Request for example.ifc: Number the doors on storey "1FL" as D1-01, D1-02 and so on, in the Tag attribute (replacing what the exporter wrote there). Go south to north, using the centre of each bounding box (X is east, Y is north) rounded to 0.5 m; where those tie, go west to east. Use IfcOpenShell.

First a look at what the model holds.

```python
import ifcopenshell
import ifcopenshell.util.element
import ifcopenshell.util.placement

model = ifcopenshell.open("example.ifc")
print(model.schema)
storey = next(s for s in model.by_type("IfcBuildingStorey") if s.Name == "1FL")
doors = [e for e in ifcopenshell.util.element.get_decomposition(storey) if e.is_a("IfcDoor")]
for e in sorted(doors, key=lambda e: e.id()):
    origin = ifcopenshell.util.placement.get_local_placement(e.ObjectPlacement)[:3, 3]
    print(e.id(), e.Tag, e.Name, origin.round(2) + 0.0, sep=" | ")
```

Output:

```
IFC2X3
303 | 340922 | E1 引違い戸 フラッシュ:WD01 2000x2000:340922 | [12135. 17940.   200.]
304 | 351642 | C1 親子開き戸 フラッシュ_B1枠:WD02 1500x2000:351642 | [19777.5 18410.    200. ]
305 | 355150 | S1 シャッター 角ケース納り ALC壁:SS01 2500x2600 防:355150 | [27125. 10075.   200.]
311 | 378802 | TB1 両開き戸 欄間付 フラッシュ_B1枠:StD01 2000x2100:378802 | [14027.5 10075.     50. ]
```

```python
import ifcopenshell
import ifcopenshell.geom
import ifcopenshell.util.element
import ifcopenshell.util.shape

model = ifcopenshell.open("example.ifc")
settings = ifcopenshell.geom.settings()
settings.set("use-world-coords", True)


def centre(element):
    shape = ifcopenshell.geom.create_shape(settings, element)
    return ifcopenshell.util.shape.get_bbox_centroid(shape.geometry)


storey = next(s for s in model.by_type("IfcBuildingStorey") if s.Name == "1FL")
doors = [e for e in ifcopenshell.util.element.get_decomposition(storey) if e.is_a("IfcDoor")]

# Insertion points can sit at a corner or the storey origin, so sort by the geometry (in metres).
centres = {e: centre(e) for e in doors}
doors.sort(key=lambda e: (round(centres[e][1] / 0.5), centres[e][0]))

for i, e in enumerate(doors, start=1):
    number = f"D1-{i:02d}"
    e.Tag = number
    print(e.id(), number)

model.write("example_updated.ifc")
```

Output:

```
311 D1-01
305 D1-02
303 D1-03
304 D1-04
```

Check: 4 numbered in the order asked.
